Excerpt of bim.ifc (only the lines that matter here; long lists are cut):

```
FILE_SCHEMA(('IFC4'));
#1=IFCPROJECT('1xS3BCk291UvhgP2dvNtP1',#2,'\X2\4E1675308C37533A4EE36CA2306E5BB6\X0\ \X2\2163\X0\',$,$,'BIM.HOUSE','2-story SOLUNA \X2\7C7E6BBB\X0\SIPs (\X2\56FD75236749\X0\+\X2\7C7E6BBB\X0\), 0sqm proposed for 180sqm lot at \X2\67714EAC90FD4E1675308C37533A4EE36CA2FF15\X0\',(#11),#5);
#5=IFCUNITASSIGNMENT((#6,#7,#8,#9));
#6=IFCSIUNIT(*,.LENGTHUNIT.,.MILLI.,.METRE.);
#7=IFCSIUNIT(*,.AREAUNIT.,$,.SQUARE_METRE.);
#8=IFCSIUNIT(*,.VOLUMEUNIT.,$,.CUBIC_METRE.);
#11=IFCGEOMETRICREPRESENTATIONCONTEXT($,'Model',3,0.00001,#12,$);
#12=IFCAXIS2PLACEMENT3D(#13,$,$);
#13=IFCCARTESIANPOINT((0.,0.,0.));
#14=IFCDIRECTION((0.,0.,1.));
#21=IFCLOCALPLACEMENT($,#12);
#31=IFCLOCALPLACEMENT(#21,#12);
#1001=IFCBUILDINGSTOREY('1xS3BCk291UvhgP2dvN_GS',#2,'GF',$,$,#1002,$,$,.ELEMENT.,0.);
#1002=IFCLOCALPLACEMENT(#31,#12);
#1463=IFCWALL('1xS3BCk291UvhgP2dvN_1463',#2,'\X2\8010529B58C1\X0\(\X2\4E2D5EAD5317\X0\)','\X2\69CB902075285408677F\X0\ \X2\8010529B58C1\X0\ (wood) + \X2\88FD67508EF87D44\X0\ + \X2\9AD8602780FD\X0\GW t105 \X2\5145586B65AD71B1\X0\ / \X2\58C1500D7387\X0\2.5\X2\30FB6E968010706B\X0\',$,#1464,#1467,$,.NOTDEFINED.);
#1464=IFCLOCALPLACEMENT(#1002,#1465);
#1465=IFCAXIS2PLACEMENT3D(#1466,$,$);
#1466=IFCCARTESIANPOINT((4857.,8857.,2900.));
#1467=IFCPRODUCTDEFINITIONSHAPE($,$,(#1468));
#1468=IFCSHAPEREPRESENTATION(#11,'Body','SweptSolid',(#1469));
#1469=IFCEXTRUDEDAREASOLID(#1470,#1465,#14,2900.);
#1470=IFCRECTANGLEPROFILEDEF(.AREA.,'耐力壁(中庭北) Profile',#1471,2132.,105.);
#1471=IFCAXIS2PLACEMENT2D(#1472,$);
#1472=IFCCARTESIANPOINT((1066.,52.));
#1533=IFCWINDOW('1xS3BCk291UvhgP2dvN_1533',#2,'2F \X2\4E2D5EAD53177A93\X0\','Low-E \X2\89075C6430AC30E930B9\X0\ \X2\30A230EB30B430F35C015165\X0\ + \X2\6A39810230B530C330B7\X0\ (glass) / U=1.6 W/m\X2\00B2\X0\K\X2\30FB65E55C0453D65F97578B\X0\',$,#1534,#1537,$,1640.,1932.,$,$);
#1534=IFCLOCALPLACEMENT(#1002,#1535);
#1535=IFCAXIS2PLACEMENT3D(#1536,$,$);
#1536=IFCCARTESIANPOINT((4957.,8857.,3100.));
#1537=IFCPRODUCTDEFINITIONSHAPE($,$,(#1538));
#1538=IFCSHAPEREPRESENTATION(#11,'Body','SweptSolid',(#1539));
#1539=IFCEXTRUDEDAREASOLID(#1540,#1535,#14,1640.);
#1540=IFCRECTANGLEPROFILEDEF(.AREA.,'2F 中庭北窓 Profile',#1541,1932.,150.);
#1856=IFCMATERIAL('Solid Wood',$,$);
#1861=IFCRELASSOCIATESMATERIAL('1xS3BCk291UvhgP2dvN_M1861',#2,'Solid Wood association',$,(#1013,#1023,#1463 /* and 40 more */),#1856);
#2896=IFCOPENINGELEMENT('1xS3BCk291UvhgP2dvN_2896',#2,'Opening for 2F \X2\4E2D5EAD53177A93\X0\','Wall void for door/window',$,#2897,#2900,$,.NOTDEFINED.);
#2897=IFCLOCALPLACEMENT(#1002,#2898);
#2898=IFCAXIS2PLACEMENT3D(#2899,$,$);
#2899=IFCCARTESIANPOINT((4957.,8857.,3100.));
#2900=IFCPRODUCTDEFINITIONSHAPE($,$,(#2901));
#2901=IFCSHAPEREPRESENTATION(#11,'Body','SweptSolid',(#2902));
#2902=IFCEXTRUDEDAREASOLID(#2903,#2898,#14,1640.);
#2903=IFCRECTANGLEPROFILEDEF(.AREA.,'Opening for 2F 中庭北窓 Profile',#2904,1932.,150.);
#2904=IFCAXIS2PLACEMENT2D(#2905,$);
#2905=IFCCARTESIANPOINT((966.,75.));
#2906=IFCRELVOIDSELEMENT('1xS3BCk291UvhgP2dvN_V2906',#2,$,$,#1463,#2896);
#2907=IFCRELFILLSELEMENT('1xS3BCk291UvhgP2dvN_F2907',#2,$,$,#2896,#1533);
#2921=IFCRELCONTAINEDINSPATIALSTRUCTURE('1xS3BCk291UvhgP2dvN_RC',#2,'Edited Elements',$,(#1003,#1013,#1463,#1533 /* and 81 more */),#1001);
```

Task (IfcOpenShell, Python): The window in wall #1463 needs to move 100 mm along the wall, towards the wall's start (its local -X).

```python
import ifcopenshell
import ifcopenshell.api.geometry
import ifcopenshell.util.placement
import ifcopenshell.util.unit

model = ifcopenshell.open("bim.ifc")
unit_scale = ifcopenshell.util.unit.calculate_unit_scale(model)

window = model.by_guid("1xS3BCk291UvhgP2dvN_1533")
opening = window.FillsVoids[0].RelatingOpeningElement
wall = opening.VoidsElements[0].RelatingBuildingElement

wall_matrix = ifcopenshell.util.placement.get_local_placement(wall.ObjectPlacement)
shift = wall_matrix[:3, 0] * -0.1 / unit_scale
before = ifcopenshell.util.placement.get_local_placement(window.ObjectPlacement)[:3, 3].copy()

# The window is not placed relative to its opening, so move both.
for product in (opening, window):
    matrix = ifcopenshell.util.placement.get_local_placement(product.ObjectPlacement)
    matrix[:3, 3] += shift
    ifcopenshell.api.geometry.edit_object_placement(model, product=product, matrix=matrix, is_si=False)

after = ifcopenshell.util.placement.get_local_placement(window.ObjectPlacement)[:3, 3]
print("window moved by", (after - before).round(3) + 0.0)

model.write("bim-out.ifc")
```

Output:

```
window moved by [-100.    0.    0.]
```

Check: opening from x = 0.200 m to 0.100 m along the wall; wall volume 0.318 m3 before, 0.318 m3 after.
